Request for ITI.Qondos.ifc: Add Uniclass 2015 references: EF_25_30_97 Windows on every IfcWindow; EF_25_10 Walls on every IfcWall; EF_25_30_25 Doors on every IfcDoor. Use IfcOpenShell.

First a look at what the model holds.

```python
import ifcopenshell

model = ifcopenshell.open("ITI.Qondos.ifc")
print(model.schema)
print("classifications:", [c.Name for c in model.by_type("IfcClassification")])
for ifc_class in ("IfcDoor", "IfcRoof", "IfcStair", "IfcWall", "IfcWindow"):
    print(ifc_class, len(model.by_type(ifc_class)))
```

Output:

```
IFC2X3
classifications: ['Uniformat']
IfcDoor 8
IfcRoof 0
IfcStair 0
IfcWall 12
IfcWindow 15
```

```python
import ifcopenshell
import ifcopenshell.api.classification

model = ifcopenshell.open("ITI.Qondos.ifc")

# IFC2X3 requires Source and Edition and has no link from the project to the system.
system = model.create_entity("IfcClassification", Source="NBS", Edition="2015", Name="Uniclass 2015")

codes = {
    "IfcWindow": ("EF_25_30_97", "Windows"),
    "IfcWall": ("EF_25_10", "Walls"),
    "IfcDoor": ("EF_25_30_25", "Doors"),
}
for ifc_class, (code, name) in codes.items():
    products = model.by_type(ifc_class)
    ifcopenshell.api.classification.add_reference(
        model, products=products, classification=system, identification=code, name=name
    )
    print(code, len(products))

model.write("ITI.Qondos_updated.ifc")
```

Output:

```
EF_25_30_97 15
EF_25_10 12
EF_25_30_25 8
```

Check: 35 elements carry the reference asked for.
